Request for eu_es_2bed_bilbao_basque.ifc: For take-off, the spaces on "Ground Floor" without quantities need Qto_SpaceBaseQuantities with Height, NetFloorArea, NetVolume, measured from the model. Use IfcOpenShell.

First a look at what the model holds.

```python
import ifcopenshell
import ifcopenshell.util.element
import ifcopenshell.util.unit

model = ifcopenshell.open("eu_es_2bed_bilbao_basque.ifc")
print(model.schema)
for unit_type in ("LENGTHUNIT", "AREAUNIT", "VOLUMEUNIT"):
    print(unit_type, ifcopenshell.util.unit.calculate_unit_scale(model, unit_type))
storey = next(s for s in model.by_type("IfcBuildingStorey") if s.Name == "Ground Floor")
spaces = [e for e in ifcopenshell.util.element.get_decomposition(storey) if e.is_a("IfcSpace")]
for e in sorted(spaces, key=lambda e: e.id()):
    print(e.id(), e.is_a(), e.Name, list(ifcopenshell.util.element.get_psets(e, qtos_only=True)), sep=" | ")
```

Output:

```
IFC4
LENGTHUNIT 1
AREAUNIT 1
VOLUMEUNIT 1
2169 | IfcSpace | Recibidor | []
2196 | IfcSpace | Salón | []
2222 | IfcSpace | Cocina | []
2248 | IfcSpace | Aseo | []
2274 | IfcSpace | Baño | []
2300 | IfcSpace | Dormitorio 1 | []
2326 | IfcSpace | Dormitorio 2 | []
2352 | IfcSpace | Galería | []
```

```python
import ifcopenshell
import ifcopenshell.api.pset
import ifcopenshell.geom
import ifcopenshell.util.element
import ifcopenshell.util.shape
import ifcopenshell.util.unit

model = ifcopenshell.open("eu_es_2bed_bilbao_basque.ifc")
unit_scale = ifcopenshell.util.unit.calculate_unit_scale(model)
area_scale = ifcopenshell.util.unit.calculate_unit_scale(model, "AREAUNIT")
volume_scale = ifcopenshell.util.unit.calculate_unit_scale(model, "VOLUMEUNIT")
settings = ifcopenshell.geom.settings()

storey = next(s for s in model.by_type("IfcBuildingStorey") if s.Name == "Ground Floor")
spaces = [e for e in ifcopenshell.util.element.get_decomposition(storey) if e.is_a("IfcSpace")]

for e in sorted(spaces, key=lambda e: e.id()):
    if ifcopenshell.util.element.get_psets(e, qtos_only=True, should_inherit=False):
        continue
    # Geometry comes back in metres, in the element's own axes.
    shape = ifcopenshell.geom.create_shape(settings, e)
    values = {
        "Height": ifcopenshell.util.shape.get_z(shape.geometry) / unit_scale,
        "NetFloorArea": ifcopenshell.util.shape.get_footprint_area(shape.geometry) / area_scale,
        "NetVolume": ifcopenshell.util.shape.get_volume(shape.geometry) / volume_scale,
    }
    qto = ifcopenshell.api.pset.add_qto(model, product=e, name="Qto_SpaceBaseQuantities")
    ifcopenshell.api.pset.edit_qto(model, qto=qto, properties=values)
    print(e.id(), {k: round(v, 3) for k, v in values.items()})

model.write("eu_es_2bed_bilbao_basque-out.ifc")
```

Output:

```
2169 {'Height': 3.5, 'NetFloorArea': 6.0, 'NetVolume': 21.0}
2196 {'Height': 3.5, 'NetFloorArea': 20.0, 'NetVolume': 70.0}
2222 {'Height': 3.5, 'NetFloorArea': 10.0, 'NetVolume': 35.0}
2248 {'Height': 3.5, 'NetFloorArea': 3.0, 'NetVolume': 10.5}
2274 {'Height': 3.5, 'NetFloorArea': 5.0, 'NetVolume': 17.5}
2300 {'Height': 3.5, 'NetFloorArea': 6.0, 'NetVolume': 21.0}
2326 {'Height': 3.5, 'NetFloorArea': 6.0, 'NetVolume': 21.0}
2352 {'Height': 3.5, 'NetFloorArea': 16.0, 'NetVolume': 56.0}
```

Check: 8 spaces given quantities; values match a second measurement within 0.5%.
